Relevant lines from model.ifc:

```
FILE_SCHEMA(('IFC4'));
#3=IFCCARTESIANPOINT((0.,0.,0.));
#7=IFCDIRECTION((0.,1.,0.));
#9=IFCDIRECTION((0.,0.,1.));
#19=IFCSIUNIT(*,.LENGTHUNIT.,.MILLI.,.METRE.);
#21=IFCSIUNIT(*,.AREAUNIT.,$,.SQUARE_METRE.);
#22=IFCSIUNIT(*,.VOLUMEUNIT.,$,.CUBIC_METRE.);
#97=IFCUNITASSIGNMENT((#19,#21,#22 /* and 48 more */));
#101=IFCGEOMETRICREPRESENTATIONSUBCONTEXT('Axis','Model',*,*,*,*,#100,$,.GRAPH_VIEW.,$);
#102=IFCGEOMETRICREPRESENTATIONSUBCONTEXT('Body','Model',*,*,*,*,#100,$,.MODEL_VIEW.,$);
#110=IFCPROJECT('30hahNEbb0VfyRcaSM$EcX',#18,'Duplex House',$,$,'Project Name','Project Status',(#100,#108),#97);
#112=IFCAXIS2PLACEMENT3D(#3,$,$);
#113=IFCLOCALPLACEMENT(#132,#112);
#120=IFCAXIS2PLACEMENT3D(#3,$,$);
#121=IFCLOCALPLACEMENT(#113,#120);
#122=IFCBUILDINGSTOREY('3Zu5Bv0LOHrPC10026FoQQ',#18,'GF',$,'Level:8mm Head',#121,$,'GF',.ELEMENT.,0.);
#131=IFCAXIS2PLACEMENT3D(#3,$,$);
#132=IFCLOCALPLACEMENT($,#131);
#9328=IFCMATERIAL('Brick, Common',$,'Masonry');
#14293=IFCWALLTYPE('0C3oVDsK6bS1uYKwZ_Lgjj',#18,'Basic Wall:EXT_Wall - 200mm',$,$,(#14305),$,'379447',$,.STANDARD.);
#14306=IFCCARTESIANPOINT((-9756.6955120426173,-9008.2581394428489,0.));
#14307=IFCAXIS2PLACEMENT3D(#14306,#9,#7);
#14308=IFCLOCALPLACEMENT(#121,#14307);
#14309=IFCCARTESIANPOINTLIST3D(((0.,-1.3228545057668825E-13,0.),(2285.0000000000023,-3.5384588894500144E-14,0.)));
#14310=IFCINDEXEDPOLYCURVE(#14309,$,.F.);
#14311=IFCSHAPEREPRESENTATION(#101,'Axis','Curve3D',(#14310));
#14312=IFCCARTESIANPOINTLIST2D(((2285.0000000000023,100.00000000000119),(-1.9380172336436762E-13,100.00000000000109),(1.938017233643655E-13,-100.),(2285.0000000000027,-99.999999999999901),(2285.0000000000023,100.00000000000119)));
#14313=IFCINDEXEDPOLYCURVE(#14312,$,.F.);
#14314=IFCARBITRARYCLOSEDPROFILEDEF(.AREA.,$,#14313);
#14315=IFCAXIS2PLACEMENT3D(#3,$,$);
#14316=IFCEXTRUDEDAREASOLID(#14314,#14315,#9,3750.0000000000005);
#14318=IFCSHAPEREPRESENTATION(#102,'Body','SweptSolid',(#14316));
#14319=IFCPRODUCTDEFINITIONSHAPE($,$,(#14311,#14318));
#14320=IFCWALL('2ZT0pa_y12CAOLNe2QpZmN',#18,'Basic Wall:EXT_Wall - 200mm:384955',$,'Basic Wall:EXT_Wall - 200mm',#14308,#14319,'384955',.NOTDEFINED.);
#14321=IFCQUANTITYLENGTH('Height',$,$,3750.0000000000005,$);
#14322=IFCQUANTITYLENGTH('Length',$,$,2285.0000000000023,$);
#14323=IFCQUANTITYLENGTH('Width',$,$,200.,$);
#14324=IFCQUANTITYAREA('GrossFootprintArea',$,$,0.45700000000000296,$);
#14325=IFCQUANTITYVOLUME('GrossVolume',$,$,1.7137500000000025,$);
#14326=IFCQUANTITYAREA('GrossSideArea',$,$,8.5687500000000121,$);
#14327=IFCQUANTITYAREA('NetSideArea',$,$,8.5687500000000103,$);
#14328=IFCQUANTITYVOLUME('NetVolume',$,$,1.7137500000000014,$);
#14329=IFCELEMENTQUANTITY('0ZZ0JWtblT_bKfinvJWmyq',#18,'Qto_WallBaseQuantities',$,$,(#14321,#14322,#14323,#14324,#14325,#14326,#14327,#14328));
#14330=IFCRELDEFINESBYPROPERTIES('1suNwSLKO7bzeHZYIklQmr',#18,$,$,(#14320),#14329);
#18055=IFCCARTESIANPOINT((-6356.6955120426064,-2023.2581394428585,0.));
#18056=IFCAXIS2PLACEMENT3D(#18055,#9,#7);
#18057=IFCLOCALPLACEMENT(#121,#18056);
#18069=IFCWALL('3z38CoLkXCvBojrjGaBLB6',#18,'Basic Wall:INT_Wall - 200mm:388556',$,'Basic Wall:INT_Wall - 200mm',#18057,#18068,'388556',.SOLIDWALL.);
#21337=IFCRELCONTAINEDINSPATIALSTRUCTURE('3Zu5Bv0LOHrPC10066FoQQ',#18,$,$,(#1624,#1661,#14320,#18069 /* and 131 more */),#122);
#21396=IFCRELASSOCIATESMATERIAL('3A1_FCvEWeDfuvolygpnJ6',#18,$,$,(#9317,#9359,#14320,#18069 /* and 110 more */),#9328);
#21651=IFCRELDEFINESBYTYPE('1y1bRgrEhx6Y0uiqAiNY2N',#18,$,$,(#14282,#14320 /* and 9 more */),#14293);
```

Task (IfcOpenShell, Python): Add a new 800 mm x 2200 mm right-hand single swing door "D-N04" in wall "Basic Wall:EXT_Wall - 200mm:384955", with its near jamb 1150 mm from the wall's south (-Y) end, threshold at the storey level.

```python
import numpy as np
import ifcopenshell
import ifcopenshell.api.feature
import ifcopenshell.api.geometry
import ifcopenshell.api.pset
import ifcopenshell.api.root
import ifcopenshell.api.spatial
import ifcopenshell.geom
import ifcopenshell.util.element
import ifcopenshell.util.placement
import ifcopenshell.util.representation
import ifcopenshell.util.shape
import ifcopenshell.util.unit

model = ifcopenshell.open("model.ifc")
unit_scale = ifcopenshell.util.unit.calculate_unit_scale(model)
area_scale = ifcopenshell.util.unit.calculate_unit_scale(model, "AREAUNIT")
volume_scale = ifcopenshell.util.unit.calculate_unit_scale(model, "VOLUMEUNIT")
settings = ifcopenshell.geom.settings()


def volume(element):
    """Net volume in cubic metres, openings subtracted."""
    shape = ifcopenshell.geom.create_shape(settings, element)
    return ifcopenshell.util.shape.get_volume(shape.geometry)


wall = model.by_guid("2ZT0pa_y12CAOLNe2QpZmN")
storey = ifcopenshell.util.element.get_container(wall, ifc_class="IfcBuildingStorey")
context = ifcopenshell.util.representation.get_context(model, "Model", "Body", "MODEL_VIEW")
before = volume(wall)

width, height, from_end, sill = 0.8, 2.2, 1.15, 0.0  # metres

# The wall runs along its own X axis, and the end named is its -X end.
wall_shape = ifcopenshell.geom.create_shape(settings, wall)
x, y, z = ifcopenshell.util.shape.get_vertices(wall_shape.geometry).T
start = x.min() + from_end
face, thickness = float(y.min()), float(y.max() - y.min())
wall_matrix = ifcopenshell.util.placement.get_local_placement(wall.ObjectPlacement)
level = ifcopenshell.util.placement.get_local_placement(storey.ObjectPlacement)[2, 3]


def in_wall(x, y):
    """Placement at x, y metres in the wall's axes, at sill height."""
    matrix = wall_matrix.copy()
    matrix[:, 3] = wall_matrix @ np.array([x / unit_scale, y / unit_scale, 0.0, 1.0])
    matrix[2, 3] = level + sill / unit_scale
    return matrix


# Opening: a box that overshoots both wall faces by 50 mm.
opening = ifcopenshell.api.root.create_entity(model, ifc_class="IfcOpeningElement", predefined_type="OPENING")
box = ifcopenshell.api.geometry.add_wall_representation(
    model, context=context, length=width, height=height, thickness=thickness + 0.1
)
ifcopenshell.api.geometry.assign_representation(model, product=opening, representation=box)
ifcopenshell.api.geometry.edit_object_placement(model, product=opening, matrix=in_wall(start, face - 0.05), is_si=False)
ifcopenshell.api.feature.add_feature(model, feature=opening, element=wall)

door = ifcopenshell.api.root.create_entity(model, ifc_class="IfcDoor", name="D-N04", predefined_type="DOOR")
door.OverallWidth, door.OverallHeight = width / unit_scale, height / unit_scale
door.OperationType = "SINGLE_SWING_RIGHT"
body = ifcopenshell.api.geometry.add_door_representation(
    model,
    context=context,
    overall_width=door.OverallWidth,
    overall_height=door.OverallHeight,
    operation_type="SINGLE_SWING_RIGHT",
    lining_properties={"LiningDepth": thickness / unit_scale, "ThresholdDepth": thickness / unit_scale},
)
ifcopenshell.api.geometry.assign_representation(model, product=door, representation=body)
ifcopenshell.api.spatial.assign_container(model, products=[door], relating_structure=storey)
ifcopenshell.api.feature.add_filling(model, opening=opening, element=door)

# The lining spans the wall, so the door starts at the wall face.
ifcopenshell.api.geometry.edit_object_placement(model, product=door, matrix=in_wall(start, face), is_si=False)

after = volume(wall)

# Update the wall's stored quantities.
qto = model.by_id(ifcopenshell.util.element.get_pset(wall, "Qto_WallBaseQuantities", should_inherit=False)["id"])
ifcopenshell.api.pset.edit_qto(model, qto=qto, properties={
    "NetSideArea": after / thickness / area_scale,
    "NetVolume": after / volume_scale,
})

print(f"wall volume {before:.3f} -> {after:.3f} m3")

model.write("model-out.ifc")
```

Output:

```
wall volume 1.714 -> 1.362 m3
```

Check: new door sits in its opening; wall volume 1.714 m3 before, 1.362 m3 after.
